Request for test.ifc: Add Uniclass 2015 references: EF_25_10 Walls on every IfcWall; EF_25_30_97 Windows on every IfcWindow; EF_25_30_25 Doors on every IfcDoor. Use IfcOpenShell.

First a look at what the model holds.

```python
import ifcopenshell

model = ifcopenshell.open("test.ifc")
print(model.schema)
print("classifications:", [c.Name for c in model.by_type("IfcClassification")])
for ifc_class in ("IfcDoor", "IfcRoof", "IfcStair", "IfcWall", "IfcWindow"):
    print(ifc_class, len(model.by_type(ifc_class)))
```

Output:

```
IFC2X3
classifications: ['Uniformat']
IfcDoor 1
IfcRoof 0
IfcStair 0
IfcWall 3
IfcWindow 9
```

```python
import ifcopenshell
import ifcopenshell.api.classification

model = ifcopenshell.open("test.ifc")

# IFC2X3 requires Source and Edition and has no link from the project to the system.
system = model.create_entity("IfcClassification", Source="NBS", Edition="2015", Name="Uniclass 2015")

codes = {
    "IfcWall": ("EF_25_10", "Walls"),
    "IfcWindow": ("EF_25_30_97", "Windows"),
    "IfcDoor": ("EF_25_30_25", "Doors"),
}
for ifc_class, (code, name) in codes.items():
    products = model.by_type(ifc_class)
    ifcopenshell.api.classification.add_reference(
        model, products=products, classification=system, identification=code, name=name
    )
    print(code, len(products))

model.write("test_v2.ifc")
```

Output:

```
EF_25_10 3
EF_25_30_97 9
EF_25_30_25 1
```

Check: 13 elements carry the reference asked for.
